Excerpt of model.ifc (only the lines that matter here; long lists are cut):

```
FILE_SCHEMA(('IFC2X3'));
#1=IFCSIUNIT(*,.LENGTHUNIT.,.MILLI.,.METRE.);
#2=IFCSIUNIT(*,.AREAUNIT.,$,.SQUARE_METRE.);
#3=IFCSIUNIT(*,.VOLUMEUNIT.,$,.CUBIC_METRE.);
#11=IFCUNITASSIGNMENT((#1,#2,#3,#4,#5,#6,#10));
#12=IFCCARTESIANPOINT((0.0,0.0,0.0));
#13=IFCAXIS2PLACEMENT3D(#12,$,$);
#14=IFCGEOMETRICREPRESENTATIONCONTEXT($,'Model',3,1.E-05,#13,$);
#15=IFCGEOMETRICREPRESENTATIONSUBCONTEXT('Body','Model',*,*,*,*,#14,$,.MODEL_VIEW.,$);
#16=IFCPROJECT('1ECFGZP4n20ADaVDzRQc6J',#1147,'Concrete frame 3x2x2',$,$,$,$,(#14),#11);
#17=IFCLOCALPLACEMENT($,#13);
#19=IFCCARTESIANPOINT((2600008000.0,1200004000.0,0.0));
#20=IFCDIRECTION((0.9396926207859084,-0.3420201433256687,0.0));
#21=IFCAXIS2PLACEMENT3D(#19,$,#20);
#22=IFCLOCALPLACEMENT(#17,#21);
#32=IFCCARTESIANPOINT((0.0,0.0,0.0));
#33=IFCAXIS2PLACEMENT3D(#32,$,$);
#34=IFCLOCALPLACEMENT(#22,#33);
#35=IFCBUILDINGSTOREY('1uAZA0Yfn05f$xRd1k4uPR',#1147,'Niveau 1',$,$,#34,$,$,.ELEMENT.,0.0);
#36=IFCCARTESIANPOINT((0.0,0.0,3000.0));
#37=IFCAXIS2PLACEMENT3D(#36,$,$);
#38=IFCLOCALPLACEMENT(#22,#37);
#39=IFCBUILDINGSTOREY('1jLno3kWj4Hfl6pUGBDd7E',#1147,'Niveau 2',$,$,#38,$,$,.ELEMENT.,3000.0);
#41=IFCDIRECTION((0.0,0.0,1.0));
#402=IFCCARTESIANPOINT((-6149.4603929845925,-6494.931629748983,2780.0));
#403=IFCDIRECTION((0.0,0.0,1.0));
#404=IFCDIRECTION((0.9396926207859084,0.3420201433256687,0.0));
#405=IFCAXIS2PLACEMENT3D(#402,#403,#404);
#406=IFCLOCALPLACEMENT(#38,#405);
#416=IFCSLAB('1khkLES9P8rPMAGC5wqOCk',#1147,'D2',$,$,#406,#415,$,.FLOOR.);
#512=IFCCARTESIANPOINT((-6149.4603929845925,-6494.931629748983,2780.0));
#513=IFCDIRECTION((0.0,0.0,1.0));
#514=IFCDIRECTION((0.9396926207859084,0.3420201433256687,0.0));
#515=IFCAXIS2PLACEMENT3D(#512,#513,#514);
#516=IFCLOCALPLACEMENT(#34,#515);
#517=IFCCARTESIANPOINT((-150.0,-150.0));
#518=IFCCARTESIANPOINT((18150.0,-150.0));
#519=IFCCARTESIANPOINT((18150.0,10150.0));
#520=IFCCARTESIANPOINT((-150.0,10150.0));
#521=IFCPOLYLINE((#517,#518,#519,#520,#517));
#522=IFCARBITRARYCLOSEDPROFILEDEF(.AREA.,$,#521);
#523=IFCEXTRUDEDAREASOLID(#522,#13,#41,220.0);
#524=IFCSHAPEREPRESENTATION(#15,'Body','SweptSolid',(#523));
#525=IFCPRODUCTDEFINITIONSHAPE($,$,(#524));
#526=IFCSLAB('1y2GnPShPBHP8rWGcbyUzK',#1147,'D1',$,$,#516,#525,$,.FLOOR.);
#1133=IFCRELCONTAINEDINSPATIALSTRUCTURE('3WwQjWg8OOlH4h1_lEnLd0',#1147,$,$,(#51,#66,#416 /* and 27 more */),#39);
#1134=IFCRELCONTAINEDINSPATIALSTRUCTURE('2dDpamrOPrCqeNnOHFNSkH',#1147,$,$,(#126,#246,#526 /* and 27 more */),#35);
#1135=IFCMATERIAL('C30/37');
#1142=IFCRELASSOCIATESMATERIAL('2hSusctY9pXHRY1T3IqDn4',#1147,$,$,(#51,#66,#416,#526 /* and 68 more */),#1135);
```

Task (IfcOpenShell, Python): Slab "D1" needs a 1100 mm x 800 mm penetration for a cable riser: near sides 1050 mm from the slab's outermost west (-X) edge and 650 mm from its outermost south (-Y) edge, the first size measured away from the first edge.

```python
import numpy as np
import ifcopenshell
import ifcopenshell.api.feature
import ifcopenshell.api.geometry
import ifcopenshell.api.root
import ifcopenshell.geom
import ifcopenshell.util.placement
import ifcopenshell.util.representation
import ifcopenshell.util.shape
import ifcopenshell.util.unit

model = ifcopenshell.open("model.ifc")
unit_scale = ifcopenshell.util.unit.calculate_unit_scale(model)
settings = ifcopenshell.geom.settings()


def volume(element):
    """Net volume in cubic metres, openings subtracted."""
    shape = ifcopenshell.geom.create_shape(settings, element)
    return ifcopenshell.util.shape.get_volume(shape.geometry)


slab = model.by_id(526)
before = volume(slab)

# Extent in the slab's own axes, in metres. The edges named are its -X and -Y sides.
slab_shape = ifcopenshell.geom.create_shape(settings, slab)
vertices = ifcopenshell.util.shape.get_vertices(slab_shape.geometry)
x_min, y_min, bottom = vertices.min(axis=0)
top = vertices[:, 2].max()

opening = ifcopenshell.api.root.create_entity(model, ifc_class="IfcOpeningElement", name="Cable riser opening")
context = ifcopenshell.util.representation.get_context(model, "Model", "Body", "MODEL_VIEW")
width, depth = 1.1, 0.8
outline = [(0.0, 0.0), (width, 0.0), (width, depth), (0.0, depth), (0.0, 0.0)]
# Overshoot both faces by 50 mm so the cut is clean.
shape = ifcopenshell.api.geometry.add_slab_representation(
    model, context=context, depth=top - bottom + 0.1, polyline=outline
)
ifcopenshell.api.geometry.assign_representation(model, product=opening, representation=shape)

matrix = ifcopenshell.util.placement.get_local_placement(slab.ObjectPlacement)
matrix[:, 3] = matrix @ np.append(np.array([x_min + 1.05, y_min + 0.65, bottom - 0.05]) / unit_scale, 1.0)
ifcopenshell.api.geometry.edit_object_placement(model, product=opening, matrix=matrix, is_si=False)
ifcopenshell.api.feature.add_feature(model, feature=opening, element=slab)

after = volume(slab)

print(f"slab volume {before:.3f} -> {after:.3f} m3")

model.write("model_v2.ifc")
```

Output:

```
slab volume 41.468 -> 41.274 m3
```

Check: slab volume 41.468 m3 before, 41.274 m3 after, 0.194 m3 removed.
